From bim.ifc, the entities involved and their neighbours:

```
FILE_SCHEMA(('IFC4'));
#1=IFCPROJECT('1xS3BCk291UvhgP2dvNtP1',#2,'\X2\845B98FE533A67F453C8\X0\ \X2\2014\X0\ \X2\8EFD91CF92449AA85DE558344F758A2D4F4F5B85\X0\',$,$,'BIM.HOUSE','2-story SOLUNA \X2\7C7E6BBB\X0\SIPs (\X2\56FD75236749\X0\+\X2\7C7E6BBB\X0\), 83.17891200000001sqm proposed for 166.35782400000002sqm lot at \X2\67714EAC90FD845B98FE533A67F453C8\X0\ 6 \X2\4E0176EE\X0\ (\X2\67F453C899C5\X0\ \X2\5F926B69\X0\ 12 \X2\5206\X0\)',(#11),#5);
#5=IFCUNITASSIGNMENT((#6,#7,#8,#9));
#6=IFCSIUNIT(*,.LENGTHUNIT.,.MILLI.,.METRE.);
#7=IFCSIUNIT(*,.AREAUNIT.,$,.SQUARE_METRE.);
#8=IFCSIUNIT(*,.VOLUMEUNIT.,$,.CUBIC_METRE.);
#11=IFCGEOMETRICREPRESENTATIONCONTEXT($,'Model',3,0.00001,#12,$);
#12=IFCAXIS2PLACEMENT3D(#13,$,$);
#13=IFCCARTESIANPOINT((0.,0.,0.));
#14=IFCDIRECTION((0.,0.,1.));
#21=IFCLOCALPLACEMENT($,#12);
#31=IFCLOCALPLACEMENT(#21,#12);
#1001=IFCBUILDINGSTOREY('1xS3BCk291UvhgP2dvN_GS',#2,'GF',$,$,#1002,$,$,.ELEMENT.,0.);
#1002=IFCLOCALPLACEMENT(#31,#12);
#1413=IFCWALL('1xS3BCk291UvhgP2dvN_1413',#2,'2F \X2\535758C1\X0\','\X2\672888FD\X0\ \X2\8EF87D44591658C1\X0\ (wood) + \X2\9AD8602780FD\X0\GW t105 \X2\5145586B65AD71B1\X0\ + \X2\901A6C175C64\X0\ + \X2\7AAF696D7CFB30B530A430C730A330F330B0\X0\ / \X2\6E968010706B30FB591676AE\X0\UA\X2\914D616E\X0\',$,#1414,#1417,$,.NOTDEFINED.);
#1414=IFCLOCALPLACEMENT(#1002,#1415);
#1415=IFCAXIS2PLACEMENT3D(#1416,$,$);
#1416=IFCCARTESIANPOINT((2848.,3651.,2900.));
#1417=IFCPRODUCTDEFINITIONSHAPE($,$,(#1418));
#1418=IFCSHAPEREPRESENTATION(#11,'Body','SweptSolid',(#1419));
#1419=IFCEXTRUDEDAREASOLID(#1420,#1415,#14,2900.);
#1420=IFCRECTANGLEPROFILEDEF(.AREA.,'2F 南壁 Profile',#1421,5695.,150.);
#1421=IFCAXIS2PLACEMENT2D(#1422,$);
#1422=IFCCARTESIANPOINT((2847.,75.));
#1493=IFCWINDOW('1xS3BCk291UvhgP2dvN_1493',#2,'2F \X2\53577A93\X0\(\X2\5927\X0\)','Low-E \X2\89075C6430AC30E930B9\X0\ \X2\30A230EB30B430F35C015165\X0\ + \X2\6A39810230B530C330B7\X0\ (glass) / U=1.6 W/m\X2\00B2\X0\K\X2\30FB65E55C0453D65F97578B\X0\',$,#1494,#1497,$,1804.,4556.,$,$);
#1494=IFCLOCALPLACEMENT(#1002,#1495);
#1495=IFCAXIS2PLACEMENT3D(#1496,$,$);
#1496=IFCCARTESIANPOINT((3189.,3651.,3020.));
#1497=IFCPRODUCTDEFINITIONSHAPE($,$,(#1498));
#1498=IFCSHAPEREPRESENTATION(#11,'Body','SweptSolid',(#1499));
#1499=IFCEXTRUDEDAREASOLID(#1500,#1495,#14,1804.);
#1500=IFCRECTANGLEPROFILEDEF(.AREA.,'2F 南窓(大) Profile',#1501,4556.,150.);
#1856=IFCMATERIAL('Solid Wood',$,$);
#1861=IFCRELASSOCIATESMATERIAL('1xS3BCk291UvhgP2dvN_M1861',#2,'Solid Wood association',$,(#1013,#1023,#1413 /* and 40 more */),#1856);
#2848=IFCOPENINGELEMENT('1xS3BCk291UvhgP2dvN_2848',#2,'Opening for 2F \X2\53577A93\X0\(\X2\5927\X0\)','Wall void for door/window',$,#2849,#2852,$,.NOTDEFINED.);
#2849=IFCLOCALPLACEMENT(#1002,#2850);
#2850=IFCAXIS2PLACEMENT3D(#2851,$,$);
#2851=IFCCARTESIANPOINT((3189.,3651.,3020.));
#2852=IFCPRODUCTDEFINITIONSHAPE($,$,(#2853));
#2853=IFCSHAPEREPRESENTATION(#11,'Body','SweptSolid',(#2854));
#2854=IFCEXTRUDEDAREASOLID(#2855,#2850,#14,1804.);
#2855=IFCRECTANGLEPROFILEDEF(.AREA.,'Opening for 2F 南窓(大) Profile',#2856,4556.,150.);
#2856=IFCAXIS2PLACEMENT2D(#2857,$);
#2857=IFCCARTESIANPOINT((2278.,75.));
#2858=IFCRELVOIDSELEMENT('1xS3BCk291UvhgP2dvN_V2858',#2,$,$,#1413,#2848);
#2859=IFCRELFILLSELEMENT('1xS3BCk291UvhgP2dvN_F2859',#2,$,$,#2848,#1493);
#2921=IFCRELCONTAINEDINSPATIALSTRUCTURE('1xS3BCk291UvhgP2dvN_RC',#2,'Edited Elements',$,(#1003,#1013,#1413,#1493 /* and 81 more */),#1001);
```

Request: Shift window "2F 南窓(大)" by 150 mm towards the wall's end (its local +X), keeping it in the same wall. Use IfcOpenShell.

```python
import ifcopenshell
import ifcopenshell.api.geometry
import ifcopenshell.util.placement

model = ifcopenshell.open("bim.ifc")

window = model.by_id(1493)
opening = window.FillsVoids[0].RelatingOpeningElement
wall = opening.VoidsElements[0].RelatingBuildingElement

wall_matrix = ifcopenshell.util.placement.get_local_placement(wall.ObjectPlacement)
shift = wall_matrix[:3, 0] * 150.0
before = ifcopenshell.util.placement.get_local_placement(window.ObjectPlacement)[:3, 3].copy()

# The window is not placed relative to its opening, so move both.
for product in (opening, window):
    matrix = ifcopenshell.util.placement.get_local_placement(product.ObjectPlacement)
    matrix[:3, 3] += shift
    ifcopenshell.api.geometry.edit_object_placement(model, product=product, matrix=matrix, is_si=False)

after = ifcopenshell.util.placement.get_local_placement(window.ObjectPlacement)[:3, 3]
print("window moved by", (after - before).round(3) + 0.0)

model.write("bim_rev.ifc")
```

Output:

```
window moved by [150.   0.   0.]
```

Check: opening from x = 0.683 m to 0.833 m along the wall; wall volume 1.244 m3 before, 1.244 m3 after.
